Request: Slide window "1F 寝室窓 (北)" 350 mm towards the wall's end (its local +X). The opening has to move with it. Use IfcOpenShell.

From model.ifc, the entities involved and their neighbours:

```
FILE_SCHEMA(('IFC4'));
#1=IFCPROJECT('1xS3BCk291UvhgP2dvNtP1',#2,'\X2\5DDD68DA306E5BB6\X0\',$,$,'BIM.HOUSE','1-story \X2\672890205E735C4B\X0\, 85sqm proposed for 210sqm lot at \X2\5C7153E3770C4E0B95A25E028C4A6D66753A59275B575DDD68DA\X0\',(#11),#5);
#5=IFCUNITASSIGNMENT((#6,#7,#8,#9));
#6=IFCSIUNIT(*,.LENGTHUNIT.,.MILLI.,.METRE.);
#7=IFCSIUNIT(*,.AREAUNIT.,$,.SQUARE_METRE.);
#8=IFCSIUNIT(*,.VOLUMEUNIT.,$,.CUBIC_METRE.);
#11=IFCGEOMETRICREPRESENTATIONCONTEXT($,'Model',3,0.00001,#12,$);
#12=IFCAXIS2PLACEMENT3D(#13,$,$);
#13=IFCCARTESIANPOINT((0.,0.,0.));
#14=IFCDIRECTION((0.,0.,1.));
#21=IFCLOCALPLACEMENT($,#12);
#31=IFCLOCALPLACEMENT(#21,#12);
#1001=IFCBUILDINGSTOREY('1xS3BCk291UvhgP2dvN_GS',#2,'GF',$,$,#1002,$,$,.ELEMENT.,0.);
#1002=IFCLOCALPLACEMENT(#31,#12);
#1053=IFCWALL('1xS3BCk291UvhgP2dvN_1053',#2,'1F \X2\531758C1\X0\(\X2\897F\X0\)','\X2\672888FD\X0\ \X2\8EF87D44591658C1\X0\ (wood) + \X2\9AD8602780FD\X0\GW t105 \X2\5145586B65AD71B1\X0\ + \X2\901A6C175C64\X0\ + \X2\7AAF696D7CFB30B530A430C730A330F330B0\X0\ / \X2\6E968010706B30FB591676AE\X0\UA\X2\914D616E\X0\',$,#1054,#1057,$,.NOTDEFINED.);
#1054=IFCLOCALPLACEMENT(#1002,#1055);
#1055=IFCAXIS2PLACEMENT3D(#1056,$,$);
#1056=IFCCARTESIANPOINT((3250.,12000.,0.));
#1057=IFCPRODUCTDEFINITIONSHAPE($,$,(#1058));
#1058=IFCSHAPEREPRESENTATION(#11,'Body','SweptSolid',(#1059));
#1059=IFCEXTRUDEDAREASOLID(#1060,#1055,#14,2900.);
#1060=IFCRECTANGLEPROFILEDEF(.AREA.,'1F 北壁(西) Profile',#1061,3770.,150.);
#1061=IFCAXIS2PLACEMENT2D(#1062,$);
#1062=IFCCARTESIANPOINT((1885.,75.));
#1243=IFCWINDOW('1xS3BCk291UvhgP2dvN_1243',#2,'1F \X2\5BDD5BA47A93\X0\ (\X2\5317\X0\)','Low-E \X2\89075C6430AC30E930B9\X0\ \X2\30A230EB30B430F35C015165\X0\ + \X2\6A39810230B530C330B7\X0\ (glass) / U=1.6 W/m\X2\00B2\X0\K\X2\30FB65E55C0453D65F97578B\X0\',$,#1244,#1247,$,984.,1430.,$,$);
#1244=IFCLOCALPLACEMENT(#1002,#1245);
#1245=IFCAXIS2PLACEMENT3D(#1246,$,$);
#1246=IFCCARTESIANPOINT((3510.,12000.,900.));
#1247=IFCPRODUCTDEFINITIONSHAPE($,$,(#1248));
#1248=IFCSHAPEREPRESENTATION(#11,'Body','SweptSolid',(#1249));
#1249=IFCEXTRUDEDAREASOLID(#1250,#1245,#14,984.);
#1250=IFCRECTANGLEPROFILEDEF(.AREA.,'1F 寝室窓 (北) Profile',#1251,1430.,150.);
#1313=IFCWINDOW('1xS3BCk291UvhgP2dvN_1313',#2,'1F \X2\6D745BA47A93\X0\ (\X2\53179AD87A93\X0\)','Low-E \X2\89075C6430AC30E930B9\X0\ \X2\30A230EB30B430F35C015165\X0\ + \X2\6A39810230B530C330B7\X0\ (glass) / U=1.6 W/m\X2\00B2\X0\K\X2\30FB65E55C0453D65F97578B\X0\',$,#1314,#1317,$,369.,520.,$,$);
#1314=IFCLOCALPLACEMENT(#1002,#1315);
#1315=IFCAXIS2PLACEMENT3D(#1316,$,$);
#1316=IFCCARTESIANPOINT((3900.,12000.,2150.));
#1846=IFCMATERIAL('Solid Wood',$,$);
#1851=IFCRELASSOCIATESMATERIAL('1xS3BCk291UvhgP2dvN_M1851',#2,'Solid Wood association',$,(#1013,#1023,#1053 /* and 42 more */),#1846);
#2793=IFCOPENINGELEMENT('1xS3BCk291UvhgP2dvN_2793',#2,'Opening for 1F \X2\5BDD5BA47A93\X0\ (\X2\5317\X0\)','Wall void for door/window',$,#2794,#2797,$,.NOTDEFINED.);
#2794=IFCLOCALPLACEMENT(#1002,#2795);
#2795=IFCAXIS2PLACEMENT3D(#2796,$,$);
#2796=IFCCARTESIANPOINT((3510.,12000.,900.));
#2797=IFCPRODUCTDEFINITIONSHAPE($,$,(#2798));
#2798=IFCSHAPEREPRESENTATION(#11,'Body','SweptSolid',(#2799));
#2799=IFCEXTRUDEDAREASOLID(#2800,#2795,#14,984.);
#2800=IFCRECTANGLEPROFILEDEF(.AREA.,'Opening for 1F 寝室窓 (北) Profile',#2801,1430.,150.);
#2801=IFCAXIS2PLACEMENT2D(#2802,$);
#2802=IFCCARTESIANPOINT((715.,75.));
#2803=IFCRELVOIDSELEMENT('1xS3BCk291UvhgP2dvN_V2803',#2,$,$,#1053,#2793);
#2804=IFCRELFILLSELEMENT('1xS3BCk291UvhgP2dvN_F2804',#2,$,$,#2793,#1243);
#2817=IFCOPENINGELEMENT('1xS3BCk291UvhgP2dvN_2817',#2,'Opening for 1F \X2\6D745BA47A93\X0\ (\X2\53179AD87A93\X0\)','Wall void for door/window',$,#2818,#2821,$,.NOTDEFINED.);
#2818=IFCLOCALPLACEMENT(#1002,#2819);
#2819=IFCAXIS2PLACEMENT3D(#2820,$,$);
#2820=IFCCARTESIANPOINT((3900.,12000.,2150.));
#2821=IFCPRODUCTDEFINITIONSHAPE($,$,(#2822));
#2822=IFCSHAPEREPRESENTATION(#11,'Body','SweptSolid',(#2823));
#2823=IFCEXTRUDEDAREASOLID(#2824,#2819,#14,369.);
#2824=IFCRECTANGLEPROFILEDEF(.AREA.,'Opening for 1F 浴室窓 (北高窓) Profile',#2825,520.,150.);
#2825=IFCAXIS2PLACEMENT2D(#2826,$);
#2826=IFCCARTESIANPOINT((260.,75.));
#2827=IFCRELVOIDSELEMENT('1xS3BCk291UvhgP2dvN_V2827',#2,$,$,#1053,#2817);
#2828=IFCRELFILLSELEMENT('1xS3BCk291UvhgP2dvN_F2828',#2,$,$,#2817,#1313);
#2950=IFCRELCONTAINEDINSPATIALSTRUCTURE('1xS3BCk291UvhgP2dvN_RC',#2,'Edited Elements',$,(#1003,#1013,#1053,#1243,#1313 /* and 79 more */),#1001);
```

```python
import ifcopenshell
import ifcopenshell.api.geometry
import ifcopenshell.util.placement

model = ifcopenshell.open("model.ifc")

window = model.by_guid("1xS3BCk291UvhgP2dvN_1243")
opening = window.FillsVoids[0].RelatingOpeningElement
wall = opening.VoidsElements[0].RelatingBuildingElement

wall_matrix = ifcopenshell.util.placement.get_local_placement(wall.ObjectPlacement)
shift = wall_matrix[:3, 0] * 350.0
before = ifcopenshell.util.placement.get_local_placement(window.ObjectPlacement)[:3, 3].copy()

# The window is not placed relative to its opening, so move both.
for product in (opening, window):
    matrix = ifcopenshell.util.placement.get_local_placement(product.ObjectPlacement)
    matrix[:3, 3] += shift
    ifcopenshell.api.geometry.edit_object_placement(model, product=product, matrix=matrix, is_si=False)

after = ifcopenshell.util.placement.get_local_placement(window.ObjectPlacement)[:3, 3]
print("window moved by", (after - before).round(3) + 0.0)

model.write("model-out.ifc")
```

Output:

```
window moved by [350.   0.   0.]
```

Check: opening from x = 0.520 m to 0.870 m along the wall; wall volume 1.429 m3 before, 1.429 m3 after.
